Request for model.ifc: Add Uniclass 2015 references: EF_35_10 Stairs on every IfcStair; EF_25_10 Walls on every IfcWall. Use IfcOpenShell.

First a look at what the model holds.

```python
import ifcopenshell

model = ifcopenshell.open("model.ifc")
print(model.schema)
print("classifications:", [c.Name for c in model.by_type("IfcClassification")])
for ifc_class in ("IfcDoor", "IfcRoof", "IfcStair", "IfcWall", "IfcWindow"):
    print(ifc_class, len(model.by_type(ifc_class)))
```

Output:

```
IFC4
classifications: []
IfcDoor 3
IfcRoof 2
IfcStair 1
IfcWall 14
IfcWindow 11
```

```python
import ifcopenshell
import ifcopenshell.api.classification

model = ifcopenshell.open("model.ifc")

system = ifcopenshell.api.classification.add_classification(model, classification="Uniclass 2015")

codes = {
    "IfcStair": ("EF_35_10", "Stairs"),
    "IfcWall": ("EF_25_10", "Walls"),
}
for ifc_class, (code, name) in codes.items():
    products = model.by_type(ifc_class)
    ifcopenshell.api.classification.add_reference(
        model, products=products, classification=system, identification=code, name=name
    )
    print(code, len(products))

model.write("model_edited.ifc")
```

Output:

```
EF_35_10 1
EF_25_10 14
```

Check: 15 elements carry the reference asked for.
